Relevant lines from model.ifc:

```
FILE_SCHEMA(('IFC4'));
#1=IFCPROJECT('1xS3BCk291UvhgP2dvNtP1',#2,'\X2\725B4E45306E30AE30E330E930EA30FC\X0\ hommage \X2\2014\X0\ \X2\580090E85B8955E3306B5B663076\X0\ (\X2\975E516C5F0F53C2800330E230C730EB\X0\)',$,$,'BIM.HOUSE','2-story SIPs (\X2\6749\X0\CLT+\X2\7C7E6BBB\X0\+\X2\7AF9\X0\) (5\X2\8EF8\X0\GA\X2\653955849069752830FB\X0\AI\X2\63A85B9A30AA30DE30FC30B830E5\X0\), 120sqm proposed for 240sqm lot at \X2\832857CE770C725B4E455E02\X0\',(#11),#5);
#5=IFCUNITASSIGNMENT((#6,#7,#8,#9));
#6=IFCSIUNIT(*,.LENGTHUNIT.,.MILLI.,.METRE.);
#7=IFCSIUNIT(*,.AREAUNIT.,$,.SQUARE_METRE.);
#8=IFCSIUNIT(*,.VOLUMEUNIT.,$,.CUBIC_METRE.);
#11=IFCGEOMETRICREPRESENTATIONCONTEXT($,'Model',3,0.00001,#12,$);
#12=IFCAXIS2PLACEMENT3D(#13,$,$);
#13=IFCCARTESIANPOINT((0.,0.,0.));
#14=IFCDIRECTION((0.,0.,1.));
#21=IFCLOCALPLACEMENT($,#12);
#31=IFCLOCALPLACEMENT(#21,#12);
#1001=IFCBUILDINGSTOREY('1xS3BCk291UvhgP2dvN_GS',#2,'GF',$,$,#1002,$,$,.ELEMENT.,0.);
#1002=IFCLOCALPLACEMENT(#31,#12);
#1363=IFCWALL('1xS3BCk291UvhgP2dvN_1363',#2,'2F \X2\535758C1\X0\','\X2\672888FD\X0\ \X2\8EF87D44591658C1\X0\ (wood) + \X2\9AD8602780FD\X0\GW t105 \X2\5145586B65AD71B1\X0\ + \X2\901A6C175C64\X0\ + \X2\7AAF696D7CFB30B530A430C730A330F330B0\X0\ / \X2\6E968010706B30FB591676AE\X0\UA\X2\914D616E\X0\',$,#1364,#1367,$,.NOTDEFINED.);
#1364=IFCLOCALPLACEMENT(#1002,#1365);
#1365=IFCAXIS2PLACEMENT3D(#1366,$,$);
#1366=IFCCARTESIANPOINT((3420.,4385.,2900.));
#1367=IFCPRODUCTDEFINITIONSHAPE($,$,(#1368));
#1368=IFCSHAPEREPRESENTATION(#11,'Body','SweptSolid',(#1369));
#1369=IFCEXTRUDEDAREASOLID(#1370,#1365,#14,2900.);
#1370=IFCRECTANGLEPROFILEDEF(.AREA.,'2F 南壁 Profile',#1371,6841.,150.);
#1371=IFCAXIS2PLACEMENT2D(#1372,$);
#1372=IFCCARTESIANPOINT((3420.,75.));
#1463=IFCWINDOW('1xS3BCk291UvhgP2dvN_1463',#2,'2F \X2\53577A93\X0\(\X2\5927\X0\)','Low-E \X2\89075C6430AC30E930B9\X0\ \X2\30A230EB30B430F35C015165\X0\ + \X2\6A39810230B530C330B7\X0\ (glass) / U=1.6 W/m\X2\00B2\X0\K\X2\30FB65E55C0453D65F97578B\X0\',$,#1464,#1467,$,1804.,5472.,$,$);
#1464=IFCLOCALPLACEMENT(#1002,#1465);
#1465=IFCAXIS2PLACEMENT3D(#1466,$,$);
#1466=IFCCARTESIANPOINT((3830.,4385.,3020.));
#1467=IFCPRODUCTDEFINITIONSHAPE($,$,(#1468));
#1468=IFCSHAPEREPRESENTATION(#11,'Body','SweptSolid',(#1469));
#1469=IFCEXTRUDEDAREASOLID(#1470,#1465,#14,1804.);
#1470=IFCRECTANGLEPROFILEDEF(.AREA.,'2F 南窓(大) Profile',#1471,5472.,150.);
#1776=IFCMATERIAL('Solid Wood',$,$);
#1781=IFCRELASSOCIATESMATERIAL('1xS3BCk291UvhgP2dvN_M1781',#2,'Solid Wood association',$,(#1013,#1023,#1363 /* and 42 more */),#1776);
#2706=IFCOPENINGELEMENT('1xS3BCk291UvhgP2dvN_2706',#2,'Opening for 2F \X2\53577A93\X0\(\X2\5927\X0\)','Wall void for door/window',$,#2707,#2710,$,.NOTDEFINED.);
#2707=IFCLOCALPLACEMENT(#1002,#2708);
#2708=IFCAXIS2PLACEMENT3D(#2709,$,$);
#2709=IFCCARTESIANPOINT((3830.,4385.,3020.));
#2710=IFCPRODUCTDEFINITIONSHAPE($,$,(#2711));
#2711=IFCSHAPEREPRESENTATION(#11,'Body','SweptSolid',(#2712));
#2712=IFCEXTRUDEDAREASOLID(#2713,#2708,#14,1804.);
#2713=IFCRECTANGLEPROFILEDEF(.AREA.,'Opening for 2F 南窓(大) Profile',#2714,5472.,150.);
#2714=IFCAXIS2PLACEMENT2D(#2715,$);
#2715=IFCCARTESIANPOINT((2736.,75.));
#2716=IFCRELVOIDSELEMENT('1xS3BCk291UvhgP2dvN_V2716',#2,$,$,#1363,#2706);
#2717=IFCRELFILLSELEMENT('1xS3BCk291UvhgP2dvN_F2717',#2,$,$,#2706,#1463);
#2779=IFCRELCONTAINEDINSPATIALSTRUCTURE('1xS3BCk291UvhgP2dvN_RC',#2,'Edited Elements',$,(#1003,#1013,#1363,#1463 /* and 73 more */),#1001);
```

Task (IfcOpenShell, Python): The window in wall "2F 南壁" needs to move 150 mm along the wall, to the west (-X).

```python
import ifcopenshell
import ifcopenshell.api.geometry
import ifcopenshell.util.placement
import ifcopenshell.util.unit

model = ifcopenshell.open("model.ifc")
unit_scale = ifcopenshell.util.unit.calculate_unit_scale(model)

window = model.by_id(1463)
opening = window.FillsVoids[0].RelatingOpeningElement
wall = opening.VoidsElements[0].RelatingBuildingElement

wall_matrix = ifcopenshell.util.placement.get_local_placement(wall.ObjectPlacement)
shift = wall_matrix[:3, 0] * -0.15 / unit_scale
before = ifcopenshell.util.placement.get_local_placement(window.ObjectPlacement)[:3, 3].copy()

# The window is not placed relative to its opening, so move both.
for product in (opening, window):
    matrix = ifcopenshell.util.placement.get_local_placement(product.ObjectPlacement)
    matrix[:3, 3] += shift
    ifcopenshell.api.geometry.edit_object_placement(model, product=product, matrix=matrix, is_si=False)

after = ifcopenshell.util.placement.get_local_placement(window.ObjectPlacement)[:3, 3]
print("window moved by", (after - before).round(3) + 0.0)

model.write("model_rev.ifc")
```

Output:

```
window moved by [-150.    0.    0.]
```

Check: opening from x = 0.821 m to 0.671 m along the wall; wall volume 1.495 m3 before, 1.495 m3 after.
